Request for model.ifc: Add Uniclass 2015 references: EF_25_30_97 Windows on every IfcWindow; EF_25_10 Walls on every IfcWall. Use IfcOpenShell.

First a look at what the model holds.

```python
import ifcopenshell

model = ifcopenshell.open("model.ifc")
print(model.schema)
print("classifications:", [c.Name for c in model.by_type("IfcClassification")])
for ifc_class in ("IfcDoor", "IfcRoof", "IfcStair", "IfcWall", "IfcWindow"):
    print(ifc_class, len(model.by_type(ifc_class)))
```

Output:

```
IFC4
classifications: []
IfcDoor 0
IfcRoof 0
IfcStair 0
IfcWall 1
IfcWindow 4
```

```python
import ifcopenshell
import ifcopenshell.api.classification

model = ifcopenshell.open("model.ifc")

system = ifcopenshell.api.classification.add_classification(model, classification="Uniclass 2015")

codes = {
    "IfcWindow": ("EF_25_30_97", "Windows"),
    "IfcWall": ("EF_25_10", "Walls"),
}
for ifc_class, (code, name) in codes.items():
    products = model.by_type(ifc_class)
    ifcopenshell.api.classification.add_reference(
        model, products=products, classification=system, identification=code, name=name
    )
    print(code, len(products))

model.write("model_rev.ifc")
```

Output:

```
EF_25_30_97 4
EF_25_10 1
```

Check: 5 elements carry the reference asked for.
